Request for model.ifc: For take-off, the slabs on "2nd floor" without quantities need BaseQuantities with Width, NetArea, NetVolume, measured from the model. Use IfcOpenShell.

First a look at what the model holds.

```python
import ifcopenshell
import ifcopenshell.util.element
import ifcopenshell.util.unit

model = ifcopenshell.open("model.ifc")
print(model.schema)
for unit_type in ("LENGTHUNIT", "AREAUNIT", "VOLUMEUNIT"):
    print(unit_type, ifcopenshell.util.unit.calculate_unit_scale(model, unit_type))
storey = next(s for s in model.by_type("IfcBuildingStorey") if s.Name == "2nd floor")
slabs = [e for e in ifcopenshell.util.element.get_decomposition(storey) if e.is_a("IfcSlab")]
for e in sorted(slabs, key=lambda e: e.id()):
    print(e.id(), e.is_a(), e.Name, list(ifcopenshell.util.element.get_psets(e, qtos_only=True)), sep=" | ")
```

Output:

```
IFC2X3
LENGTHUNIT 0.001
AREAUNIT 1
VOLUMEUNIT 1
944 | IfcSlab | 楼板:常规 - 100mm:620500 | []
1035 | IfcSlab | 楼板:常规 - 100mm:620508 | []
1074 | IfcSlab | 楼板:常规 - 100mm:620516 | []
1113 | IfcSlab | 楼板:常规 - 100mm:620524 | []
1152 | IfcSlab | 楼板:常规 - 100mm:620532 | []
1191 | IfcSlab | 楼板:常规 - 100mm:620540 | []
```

```python
import ifcopenshell
import ifcopenshell.api.pset
import ifcopenshell.geom
import ifcopenshell.util.element
import ifcopenshell.util.shape
import ifcopenshell.util.unit

model = ifcopenshell.open("model.ifc")
unit_scale = ifcopenshell.util.unit.calculate_unit_scale(model)
area_scale = ifcopenshell.util.unit.calculate_unit_scale(model, "AREAUNIT")
volume_scale = ifcopenshell.util.unit.calculate_unit_scale(model, "VOLUMEUNIT")
settings = ifcopenshell.geom.settings()

storey = next(s for s in model.by_type("IfcBuildingStorey") if s.Name == "2nd floor")
slabs = [e for e in ifcopenshell.util.element.get_decomposition(storey) if e.is_a("IfcSlab")]

for e in sorted(slabs, key=lambda e: e.id()):
    if ifcopenshell.util.element.get_psets(e, qtos_only=True, should_inherit=False):
        continue
    # Geometry comes back in metres, in the element's own axes.
    shape = ifcopenshell.geom.create_shape(settings, e)
    values = {
        "Width": ifcopenshell.util.shape.get_z(shape.geometry) / unit_scale,
        "NetArea": ifcopenshell.util.shape.get_footprint_area(shape.geometry) / area_scale,
        "NetVolume": ifcopenshell.util.shape.get_volume(shape.geometry) / volume_scale,
    }
    qto = ifcopenshell.api.pset.add_qto(model, product=e, name="BaseQuantities")
    ifcopenshell.api.pset.edit_qto(model, qto=qto, properties=values)
    print(e.id(), {k: round(v, 3) for k, v in values.items()})

model.write("model_v2.ifc")
```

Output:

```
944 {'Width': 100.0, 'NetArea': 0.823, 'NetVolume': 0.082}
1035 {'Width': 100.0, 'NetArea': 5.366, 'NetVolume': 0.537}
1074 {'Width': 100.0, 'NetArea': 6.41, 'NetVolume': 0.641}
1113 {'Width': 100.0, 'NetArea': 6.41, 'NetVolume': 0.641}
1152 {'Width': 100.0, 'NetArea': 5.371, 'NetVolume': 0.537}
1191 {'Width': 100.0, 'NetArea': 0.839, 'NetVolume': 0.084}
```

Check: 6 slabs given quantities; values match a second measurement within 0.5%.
